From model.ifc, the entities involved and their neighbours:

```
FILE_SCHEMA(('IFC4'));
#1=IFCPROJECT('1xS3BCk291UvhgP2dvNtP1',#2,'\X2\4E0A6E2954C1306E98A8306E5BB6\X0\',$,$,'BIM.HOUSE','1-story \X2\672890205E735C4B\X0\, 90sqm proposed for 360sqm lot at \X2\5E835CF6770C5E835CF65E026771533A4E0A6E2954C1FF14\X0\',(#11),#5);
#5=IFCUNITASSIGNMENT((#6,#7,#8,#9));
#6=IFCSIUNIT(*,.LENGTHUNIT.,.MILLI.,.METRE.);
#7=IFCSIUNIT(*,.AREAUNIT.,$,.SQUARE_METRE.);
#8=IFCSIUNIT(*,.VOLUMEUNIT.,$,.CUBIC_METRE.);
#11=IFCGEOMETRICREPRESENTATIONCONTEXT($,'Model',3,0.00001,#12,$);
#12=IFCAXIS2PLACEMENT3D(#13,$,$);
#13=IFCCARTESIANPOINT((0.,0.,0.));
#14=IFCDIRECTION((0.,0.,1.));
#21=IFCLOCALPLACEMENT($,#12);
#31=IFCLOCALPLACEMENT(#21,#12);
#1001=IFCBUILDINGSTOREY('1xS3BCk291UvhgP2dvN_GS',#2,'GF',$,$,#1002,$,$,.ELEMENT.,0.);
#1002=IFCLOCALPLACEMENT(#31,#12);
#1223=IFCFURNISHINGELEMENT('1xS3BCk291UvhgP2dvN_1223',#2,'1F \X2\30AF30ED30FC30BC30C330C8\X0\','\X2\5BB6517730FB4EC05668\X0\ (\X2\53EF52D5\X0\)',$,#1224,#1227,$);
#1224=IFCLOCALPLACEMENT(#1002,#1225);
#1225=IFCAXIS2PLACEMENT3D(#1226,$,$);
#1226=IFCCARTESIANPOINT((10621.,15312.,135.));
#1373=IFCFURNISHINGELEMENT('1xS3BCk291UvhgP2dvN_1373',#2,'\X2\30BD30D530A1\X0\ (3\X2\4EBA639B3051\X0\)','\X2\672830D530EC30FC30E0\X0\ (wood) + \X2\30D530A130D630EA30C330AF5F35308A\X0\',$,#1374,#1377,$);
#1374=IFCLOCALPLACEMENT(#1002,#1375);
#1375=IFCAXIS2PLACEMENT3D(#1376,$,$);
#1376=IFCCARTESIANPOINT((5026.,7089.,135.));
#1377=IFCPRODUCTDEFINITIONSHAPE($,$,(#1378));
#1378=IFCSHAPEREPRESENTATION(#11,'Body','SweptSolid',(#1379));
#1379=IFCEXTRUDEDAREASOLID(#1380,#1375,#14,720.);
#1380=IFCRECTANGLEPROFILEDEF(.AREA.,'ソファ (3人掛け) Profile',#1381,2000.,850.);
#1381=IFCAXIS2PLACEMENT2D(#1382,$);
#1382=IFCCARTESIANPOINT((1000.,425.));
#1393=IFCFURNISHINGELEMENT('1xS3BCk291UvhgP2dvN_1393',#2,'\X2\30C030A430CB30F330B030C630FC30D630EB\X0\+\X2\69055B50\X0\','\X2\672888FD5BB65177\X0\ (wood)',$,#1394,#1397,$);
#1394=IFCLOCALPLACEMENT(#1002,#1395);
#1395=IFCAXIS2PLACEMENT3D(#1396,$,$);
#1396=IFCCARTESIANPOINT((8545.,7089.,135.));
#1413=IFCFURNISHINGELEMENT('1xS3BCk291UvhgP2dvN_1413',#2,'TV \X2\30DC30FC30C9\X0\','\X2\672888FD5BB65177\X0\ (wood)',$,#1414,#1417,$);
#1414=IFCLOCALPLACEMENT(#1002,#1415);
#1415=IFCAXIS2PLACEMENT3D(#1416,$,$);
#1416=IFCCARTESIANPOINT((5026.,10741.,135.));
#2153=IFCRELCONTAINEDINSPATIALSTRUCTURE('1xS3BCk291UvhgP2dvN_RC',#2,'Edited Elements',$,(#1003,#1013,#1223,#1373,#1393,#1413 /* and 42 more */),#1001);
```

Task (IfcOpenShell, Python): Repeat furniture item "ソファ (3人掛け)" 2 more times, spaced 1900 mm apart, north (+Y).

```python
import numpy as np
import ifcopenshell
import ifcopenshell.api.geometry
import ifcopenshell.api.root
import ifcopenshell.util.element
import ifcopenshell.util.placement

model = ifcopenshell.open("model.ifc")


def reuse_history(source, copy):
    """copy_class also copies each property set's owner history, people and application; keep the originals."""
    for rel in copy.IsDefinedBy:
        if rel.is_a("IfcRelDefinesByProperties") and (history := rel.RelatingPropertyDefinition.OwnerHistory):
            rel.RelatingPropertyDefinition.OwnerHistory = source.OwnerHistory
            ifcopenshell.util.element.remove_deep2(model, history)


source = model.by_id(1373)
base = ifcopenshell.util.placement.get_local_placement(source.ObjectPlacement)
step = np.array([0.0, 1.0, 0.0]) * 1900.0

for i in range(1, 3):
    copy = ifcopenshell.api.root.copy_class(model, product=source)
    copy.Representation = ifcopenshell.util.element.copy_deep(
        model, source.Representation, exclude=["IfcGeometricRepresentationContext", "IfcRepresentationMap"]
    )
    reuse_history(source, copy)
    matrix = base.copy()
    matrix[:3, 3] += i * step
    print("added at", matrix[:3, 3].round(3) + 0.0)
    ifcopenshell.api.geometry.edit_object_placement(model, product=copy, matrix=matrix, is_si=False)

model.write("model-out.ifc")
```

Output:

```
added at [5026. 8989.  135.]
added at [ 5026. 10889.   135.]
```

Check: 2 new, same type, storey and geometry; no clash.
